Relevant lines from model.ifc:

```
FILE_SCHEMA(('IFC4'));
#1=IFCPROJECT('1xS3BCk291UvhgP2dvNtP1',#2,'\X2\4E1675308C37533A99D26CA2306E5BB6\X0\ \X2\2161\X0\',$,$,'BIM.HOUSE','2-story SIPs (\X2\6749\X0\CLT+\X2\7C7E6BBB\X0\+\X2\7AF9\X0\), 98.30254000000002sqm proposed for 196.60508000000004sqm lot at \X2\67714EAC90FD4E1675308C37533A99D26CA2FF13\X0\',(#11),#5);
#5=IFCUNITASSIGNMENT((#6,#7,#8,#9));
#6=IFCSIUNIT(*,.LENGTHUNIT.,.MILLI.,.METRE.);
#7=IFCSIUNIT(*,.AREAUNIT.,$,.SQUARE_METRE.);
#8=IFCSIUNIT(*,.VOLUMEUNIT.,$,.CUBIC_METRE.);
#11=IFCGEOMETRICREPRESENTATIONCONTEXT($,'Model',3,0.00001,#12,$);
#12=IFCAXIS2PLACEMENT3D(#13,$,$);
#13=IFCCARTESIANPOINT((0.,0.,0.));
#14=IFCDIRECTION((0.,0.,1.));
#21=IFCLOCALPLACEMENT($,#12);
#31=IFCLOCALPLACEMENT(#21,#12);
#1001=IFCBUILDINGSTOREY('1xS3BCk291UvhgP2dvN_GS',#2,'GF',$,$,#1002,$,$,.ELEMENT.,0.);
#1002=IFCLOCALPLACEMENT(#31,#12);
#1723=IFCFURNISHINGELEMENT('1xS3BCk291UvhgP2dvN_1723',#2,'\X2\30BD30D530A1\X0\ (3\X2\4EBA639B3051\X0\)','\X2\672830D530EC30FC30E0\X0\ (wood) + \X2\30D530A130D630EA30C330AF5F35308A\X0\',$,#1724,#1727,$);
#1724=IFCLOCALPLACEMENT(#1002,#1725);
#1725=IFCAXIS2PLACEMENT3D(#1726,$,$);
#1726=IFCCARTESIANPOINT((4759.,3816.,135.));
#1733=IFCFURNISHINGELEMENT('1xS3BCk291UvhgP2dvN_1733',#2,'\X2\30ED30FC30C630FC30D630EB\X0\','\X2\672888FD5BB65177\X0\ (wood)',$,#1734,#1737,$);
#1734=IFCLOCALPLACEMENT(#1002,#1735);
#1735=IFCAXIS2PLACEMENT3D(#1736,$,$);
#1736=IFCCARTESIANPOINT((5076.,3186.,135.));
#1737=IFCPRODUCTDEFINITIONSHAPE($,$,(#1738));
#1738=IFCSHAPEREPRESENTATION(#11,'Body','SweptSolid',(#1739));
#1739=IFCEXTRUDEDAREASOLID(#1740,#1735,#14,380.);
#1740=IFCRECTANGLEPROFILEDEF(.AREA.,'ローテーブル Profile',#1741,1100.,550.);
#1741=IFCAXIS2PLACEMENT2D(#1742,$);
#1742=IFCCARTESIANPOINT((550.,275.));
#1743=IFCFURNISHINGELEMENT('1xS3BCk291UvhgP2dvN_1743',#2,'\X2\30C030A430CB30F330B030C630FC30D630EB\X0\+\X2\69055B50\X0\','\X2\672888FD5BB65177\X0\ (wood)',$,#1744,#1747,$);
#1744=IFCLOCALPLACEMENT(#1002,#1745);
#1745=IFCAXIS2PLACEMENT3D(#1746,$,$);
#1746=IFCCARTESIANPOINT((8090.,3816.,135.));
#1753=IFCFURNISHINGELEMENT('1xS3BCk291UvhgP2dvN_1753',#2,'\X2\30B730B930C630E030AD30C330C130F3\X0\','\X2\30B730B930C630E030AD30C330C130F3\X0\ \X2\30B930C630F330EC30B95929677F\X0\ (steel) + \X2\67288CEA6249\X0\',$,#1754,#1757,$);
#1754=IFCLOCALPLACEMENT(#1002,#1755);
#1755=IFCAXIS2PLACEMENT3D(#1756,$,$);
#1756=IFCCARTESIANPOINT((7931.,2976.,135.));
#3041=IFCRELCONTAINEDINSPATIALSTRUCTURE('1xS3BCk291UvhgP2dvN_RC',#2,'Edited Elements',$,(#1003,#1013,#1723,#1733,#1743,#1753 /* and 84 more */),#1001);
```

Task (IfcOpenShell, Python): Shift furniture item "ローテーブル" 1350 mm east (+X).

```python
import ifcopenshell
import ifcopenshell.api.geometry
import ifcopenshell.util.placement

model = ifcopenshell.open("model.ifc")

item = model.by_guid("1xS3BCk291UvhgP2dvN_1733")
matrix = ifcopenshell.util.placement.get_local_placement(item.ObjectPlacement)
matrix[0, 3] += 1350.0
ifcopenshell.api.geometry.edit_object_placement(model, product=item, matrix=matrix, is_si=False)

print(ifcopenshell.util.placement.get_local_placement(item.ObjectPlacement).round(3) + 0.0)

model.write("model_v2.ifc")
```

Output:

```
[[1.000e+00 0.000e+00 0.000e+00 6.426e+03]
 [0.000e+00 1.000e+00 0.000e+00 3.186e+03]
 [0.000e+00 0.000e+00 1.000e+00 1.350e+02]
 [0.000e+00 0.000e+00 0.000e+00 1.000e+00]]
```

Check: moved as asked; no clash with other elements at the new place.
